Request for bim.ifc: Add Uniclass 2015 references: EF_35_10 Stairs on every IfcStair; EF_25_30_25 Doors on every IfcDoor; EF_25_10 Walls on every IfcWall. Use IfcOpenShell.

First a look at what the model holds.

```python
import ifcopenshell

model = ifcopenshell.open("bim.ifc")
print(model.schema)
print("classifications:", [c.Name for c in model.by_type("IfcClassification")])
for ifc_class in ("IfcDoor", "IfcRoof", "IfcStair", "IfcWall", "IfcWindow"):
    print(ifc_class, len(model.by_type(ifc_class)))
```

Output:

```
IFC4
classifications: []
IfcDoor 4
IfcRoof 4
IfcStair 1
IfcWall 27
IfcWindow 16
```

```python
import ifcopenshell
import ifcopenshell.api.classification

model = ifcopenshell.open("bim.ifc")

system = ifcopenshell.api.classification.add_classification(model, classification="Uniclass 2015")

codes = {
    "IfcStair": ("EF_35_10", "Stairs"),
    "IfcDoor": ("EF_25_30_25", "Doors"),
    "IfcWall": ("EF_25_10", "Walls"),
}
for ifc_class, (code, name) in codes.items():
    products = model.by_type(ifc_class)
    ifcopenshell.api.classification.add_reference(
        model, products=products, classification=system, identification=code, name=name
    )
    print(code, len(products))

model.write("bim_edited.ifc")
```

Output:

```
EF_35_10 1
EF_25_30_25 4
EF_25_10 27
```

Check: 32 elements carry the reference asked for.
